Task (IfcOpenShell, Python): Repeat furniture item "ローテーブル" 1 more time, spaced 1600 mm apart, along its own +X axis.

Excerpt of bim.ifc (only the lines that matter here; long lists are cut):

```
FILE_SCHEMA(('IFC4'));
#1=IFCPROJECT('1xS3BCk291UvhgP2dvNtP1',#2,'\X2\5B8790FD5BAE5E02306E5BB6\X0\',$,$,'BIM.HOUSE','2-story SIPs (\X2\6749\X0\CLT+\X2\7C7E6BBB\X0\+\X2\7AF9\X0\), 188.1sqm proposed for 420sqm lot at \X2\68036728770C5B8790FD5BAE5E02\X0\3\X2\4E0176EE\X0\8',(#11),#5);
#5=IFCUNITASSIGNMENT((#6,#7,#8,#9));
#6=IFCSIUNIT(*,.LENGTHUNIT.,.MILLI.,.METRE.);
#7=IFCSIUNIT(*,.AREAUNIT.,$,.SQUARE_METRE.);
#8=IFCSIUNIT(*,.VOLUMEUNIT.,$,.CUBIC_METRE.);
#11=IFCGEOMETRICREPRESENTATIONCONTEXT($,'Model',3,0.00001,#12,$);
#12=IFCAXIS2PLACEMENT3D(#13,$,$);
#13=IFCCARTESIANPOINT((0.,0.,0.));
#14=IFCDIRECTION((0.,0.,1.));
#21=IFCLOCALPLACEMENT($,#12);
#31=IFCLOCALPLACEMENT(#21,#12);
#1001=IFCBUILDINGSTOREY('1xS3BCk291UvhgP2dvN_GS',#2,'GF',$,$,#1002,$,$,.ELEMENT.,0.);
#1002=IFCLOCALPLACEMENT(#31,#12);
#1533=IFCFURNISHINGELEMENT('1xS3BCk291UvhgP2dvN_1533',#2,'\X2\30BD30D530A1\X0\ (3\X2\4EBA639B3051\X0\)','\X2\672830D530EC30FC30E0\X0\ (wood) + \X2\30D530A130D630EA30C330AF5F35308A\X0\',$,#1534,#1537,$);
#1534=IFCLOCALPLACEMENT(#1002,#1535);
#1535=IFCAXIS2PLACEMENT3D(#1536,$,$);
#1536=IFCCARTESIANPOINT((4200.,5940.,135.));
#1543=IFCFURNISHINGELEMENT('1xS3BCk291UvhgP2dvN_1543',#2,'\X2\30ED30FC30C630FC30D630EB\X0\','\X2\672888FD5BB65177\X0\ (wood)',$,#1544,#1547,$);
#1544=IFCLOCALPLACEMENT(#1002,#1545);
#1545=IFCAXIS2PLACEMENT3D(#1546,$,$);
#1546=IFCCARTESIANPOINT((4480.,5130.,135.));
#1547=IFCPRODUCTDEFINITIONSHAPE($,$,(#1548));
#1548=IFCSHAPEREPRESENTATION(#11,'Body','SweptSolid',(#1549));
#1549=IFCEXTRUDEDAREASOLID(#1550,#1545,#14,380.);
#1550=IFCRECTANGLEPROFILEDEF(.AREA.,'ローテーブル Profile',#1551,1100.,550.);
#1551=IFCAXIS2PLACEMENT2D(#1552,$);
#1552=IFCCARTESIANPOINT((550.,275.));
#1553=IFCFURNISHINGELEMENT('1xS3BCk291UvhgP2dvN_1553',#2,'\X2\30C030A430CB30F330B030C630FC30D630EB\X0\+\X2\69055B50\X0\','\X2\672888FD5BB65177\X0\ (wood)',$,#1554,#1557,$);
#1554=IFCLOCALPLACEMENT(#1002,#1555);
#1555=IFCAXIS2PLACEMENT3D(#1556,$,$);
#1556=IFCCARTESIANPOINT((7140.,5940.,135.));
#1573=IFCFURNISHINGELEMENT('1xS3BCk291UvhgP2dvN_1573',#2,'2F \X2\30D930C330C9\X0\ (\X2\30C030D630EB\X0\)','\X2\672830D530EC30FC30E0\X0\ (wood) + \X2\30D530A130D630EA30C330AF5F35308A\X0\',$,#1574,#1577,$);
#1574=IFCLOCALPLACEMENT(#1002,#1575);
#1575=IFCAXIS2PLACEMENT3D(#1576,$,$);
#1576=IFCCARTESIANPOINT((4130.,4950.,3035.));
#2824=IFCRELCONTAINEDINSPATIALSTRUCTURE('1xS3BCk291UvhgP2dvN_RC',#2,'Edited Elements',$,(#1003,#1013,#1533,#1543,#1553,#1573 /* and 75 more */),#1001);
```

```python
import ifcopenshell
import ifcopenshell.api.geometry
import ifcopenshell.api.root
import ifcopenshell.util.element
import ifcopenshell.util.placement
import ifcopenshell.util.unit

model = ifcopenshell.open("bim.ifc")
unit_scale = ifcopenshell.util.unit.calculate_unit_scale(model)


def reuse_history(source, copy):
    """copy_class also copies each property set's owner history, people and application; keep the originals."""
    for rel in copy.IsDefinedBy:
        if rel.is_a("IfcRelDefinesByProperties") and (history := rel.RelatingPropertyDefinition.OwnerHistory):
            rel.RelatingPropertyDefinition.OwnerHistory = source.OwnerHistory
            ifcopenshell.util.element.remove_deep2(model, history)


source = model.by_id(1543)
base = ifcopenshell.util.placement.get_local_placement(source.ObjectPlacement)
step = base[:3, 0] * 1.6 / unit_scale

for i in range(1, 2):
    copy = ifcopenshell.api.root.copy_class(model, product=source)
    copy.Representation = ifcopenshell.util.element.copy_deep(
        model, source.Representation, exclude=["IfcGeometricRepresentationContext", "IfcRepresentationMap"]
    )
    reuse_history(source, copy)
    matrix = base.copy()
    matrix[:3, 3] += i * step
    print("added at", matrix[:3, 3].round(3) + 0.0)
    ifcopenshell.api.geometry.edit_object_placement(model, product=copy, matrix=matrix, is_si=False)

model.write("bim-out.ifc")
```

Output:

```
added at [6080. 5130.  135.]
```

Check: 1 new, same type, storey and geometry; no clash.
